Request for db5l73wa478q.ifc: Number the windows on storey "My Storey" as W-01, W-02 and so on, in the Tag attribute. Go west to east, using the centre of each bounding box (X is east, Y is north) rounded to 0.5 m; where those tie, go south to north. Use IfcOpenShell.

First a look at what the model holds.

```python
import ifcopenshell
import ifcopenshell.util.element
import ifcopenshell.util.placement

model = ifcopenshell.open("db5l73wa478q.ifc")
print(model.schema)
storey = next(s for s in model.by_type("IfcBuildingStorey") if s.Name == "My Storey")
windows = [e for e in ifcopenshell.util.element.get_decomposition(storey) if e.is_a("IfcWindow")]
for e in sorted(windows, key=lambda e: e.id()):
    origin = ifcopenshell.util.placement.get_local_placement(e.ObjectPlacement)[:3, 3]
    print(e.id(), e.Tag, e.Name, origin.round(2) + 0.0, sep=" | ")
```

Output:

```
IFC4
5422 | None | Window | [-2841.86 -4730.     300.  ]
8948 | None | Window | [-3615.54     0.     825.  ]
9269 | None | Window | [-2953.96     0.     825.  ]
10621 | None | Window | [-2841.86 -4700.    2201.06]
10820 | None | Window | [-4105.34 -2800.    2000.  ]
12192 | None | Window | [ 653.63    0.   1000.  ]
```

```python
import ifcopenshell
import ifcopenshell.geom
import ifcopenshell.util.element
import ifcopenshell.util.shape

model = ifcopenshell.open("db5l73wa478q.ifc")
settings = ifcopenshell.geom.settings()
settings.set("use-world-coords", True)


def centre(element):
    shape = ifcopenshell.geom.create_shape(settings, element)
    return ifcopenshell.util.shape.get_bbox_centroid(shape.geometry)


storey = next(s for s in model.by_type("IfcBuildingStorey") if s.Name == "My Storey")
windows = [e for e in ifcopenshell.util.element.get_decomposition(storey) if e.is_a("IfcWindow")]

# Insertion points can sit at a corner or the storey origin, so sort by the geometry (in metres).
centres = {e: centre(e) for e in windows}
windows.sort(key=lambda e: (round(centres[e][0] / 0.5), centres[e][1]))

for i, e in enumerate(windows, start=1):
    number = f"W-{i:02d}"
    e.Tag = number
    print(e.id(), number)

model.write("db5l73wa478q-out.ifc")
```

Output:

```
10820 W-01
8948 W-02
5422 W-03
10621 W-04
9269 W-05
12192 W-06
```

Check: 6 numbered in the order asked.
